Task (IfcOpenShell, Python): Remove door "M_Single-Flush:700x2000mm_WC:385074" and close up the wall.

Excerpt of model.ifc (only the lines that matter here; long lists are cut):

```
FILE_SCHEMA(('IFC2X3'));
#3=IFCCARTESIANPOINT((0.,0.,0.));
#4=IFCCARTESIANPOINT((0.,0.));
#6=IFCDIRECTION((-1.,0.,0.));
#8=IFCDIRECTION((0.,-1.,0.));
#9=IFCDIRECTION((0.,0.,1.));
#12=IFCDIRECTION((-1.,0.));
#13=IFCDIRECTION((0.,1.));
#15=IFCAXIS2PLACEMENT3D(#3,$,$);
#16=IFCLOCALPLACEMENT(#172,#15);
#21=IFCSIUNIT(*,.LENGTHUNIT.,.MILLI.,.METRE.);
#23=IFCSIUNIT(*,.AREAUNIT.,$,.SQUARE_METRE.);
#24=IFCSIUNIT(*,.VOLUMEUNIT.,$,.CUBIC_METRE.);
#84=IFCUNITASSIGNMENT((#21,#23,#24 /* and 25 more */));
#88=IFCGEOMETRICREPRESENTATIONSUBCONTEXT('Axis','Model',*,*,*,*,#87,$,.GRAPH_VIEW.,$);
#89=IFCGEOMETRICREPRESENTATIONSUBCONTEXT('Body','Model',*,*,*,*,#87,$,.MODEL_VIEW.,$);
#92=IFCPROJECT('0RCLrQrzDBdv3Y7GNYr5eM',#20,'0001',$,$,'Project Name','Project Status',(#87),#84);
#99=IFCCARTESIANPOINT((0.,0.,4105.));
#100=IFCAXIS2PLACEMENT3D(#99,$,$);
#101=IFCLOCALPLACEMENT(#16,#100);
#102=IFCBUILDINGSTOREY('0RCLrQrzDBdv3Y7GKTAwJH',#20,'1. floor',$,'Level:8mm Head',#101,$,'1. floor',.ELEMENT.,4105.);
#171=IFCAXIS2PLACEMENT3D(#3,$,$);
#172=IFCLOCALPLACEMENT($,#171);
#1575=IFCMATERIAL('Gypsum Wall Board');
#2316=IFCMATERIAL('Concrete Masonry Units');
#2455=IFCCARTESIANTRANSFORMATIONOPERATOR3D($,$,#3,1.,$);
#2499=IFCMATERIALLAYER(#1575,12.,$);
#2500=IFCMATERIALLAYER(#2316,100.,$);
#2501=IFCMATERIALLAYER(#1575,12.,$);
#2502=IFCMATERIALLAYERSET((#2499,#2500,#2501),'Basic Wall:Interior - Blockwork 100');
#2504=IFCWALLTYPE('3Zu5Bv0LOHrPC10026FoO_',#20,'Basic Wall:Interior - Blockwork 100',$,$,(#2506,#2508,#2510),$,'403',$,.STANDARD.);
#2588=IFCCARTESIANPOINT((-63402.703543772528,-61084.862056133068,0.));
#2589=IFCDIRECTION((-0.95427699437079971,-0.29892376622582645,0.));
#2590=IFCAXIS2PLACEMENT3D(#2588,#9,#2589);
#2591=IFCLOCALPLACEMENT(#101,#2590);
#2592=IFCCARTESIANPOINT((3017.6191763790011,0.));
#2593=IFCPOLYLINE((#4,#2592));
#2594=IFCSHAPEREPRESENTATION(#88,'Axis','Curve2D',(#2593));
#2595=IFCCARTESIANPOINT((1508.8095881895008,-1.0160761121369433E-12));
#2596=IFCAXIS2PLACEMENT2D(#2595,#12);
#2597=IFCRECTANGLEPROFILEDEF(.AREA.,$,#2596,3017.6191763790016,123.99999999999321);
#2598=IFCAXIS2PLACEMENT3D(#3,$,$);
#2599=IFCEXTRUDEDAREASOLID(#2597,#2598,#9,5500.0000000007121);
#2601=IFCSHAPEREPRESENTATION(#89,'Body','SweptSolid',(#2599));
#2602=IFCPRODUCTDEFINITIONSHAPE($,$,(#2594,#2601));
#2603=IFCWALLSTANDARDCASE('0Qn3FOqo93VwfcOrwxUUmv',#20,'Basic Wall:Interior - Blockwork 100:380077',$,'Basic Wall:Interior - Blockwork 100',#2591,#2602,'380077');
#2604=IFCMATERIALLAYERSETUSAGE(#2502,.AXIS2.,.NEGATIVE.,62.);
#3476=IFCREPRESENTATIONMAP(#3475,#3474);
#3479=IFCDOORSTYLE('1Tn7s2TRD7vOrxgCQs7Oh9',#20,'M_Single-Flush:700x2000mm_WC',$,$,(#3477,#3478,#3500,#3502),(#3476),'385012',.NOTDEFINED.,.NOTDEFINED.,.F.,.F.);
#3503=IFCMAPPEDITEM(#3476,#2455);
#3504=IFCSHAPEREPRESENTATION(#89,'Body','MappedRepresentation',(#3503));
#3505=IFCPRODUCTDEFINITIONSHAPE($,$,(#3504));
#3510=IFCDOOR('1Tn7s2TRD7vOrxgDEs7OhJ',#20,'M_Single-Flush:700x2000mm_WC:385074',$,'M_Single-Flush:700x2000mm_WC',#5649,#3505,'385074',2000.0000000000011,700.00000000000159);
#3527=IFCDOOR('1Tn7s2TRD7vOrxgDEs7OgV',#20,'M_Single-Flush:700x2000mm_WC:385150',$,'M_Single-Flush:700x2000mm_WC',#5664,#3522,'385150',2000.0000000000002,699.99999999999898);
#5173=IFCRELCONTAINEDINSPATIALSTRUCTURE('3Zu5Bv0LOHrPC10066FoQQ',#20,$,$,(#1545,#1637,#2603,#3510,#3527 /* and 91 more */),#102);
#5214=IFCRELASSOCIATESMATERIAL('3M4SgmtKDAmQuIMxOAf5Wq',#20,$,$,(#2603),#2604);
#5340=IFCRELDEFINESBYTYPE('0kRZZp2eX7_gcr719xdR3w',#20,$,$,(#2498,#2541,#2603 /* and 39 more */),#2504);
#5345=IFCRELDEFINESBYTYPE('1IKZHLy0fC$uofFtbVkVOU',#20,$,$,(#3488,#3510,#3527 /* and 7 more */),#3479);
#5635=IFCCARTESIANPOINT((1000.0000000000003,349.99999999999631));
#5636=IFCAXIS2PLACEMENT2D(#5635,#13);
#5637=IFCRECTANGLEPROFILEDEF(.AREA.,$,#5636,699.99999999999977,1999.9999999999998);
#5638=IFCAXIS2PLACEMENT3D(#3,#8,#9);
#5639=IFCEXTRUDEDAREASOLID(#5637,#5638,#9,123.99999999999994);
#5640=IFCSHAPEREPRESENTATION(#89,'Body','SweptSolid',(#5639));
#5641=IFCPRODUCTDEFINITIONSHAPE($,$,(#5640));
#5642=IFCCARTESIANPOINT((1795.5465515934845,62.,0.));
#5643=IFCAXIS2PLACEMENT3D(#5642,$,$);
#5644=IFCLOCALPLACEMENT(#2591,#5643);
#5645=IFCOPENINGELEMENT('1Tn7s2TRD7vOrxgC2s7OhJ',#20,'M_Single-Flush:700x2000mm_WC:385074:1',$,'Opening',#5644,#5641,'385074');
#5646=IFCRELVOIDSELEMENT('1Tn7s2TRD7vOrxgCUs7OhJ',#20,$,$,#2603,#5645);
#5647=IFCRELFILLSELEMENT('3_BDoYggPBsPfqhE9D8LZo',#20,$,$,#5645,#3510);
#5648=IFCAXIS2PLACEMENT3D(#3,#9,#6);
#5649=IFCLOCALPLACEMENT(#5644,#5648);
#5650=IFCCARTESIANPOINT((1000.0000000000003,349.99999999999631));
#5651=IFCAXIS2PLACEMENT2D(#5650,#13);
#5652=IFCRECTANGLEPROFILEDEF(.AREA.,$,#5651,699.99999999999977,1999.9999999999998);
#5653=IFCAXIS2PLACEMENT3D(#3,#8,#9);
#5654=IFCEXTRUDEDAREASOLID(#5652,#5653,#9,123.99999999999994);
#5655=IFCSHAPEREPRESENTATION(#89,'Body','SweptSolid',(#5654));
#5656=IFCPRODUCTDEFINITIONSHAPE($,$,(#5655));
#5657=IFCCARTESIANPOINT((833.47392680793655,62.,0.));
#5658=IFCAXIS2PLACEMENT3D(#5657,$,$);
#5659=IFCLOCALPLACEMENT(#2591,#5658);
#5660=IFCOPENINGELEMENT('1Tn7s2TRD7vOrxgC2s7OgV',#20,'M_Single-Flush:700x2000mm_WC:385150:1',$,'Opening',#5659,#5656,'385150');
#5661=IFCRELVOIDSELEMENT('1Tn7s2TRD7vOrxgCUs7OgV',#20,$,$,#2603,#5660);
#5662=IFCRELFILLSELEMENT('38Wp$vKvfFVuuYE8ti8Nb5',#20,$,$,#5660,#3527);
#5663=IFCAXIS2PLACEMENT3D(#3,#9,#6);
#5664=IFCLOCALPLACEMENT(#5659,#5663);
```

```python
import ifcopenshell
import ifcopenshell.api.feature
import ifcopenshell.api.root
import ifcopenshell.geom
import ifcopenshell.util.shape

model = ifcopenshell.open("model.ifc")
settings = ifcopenshell.geom.settings()


def volume(element):
    """Net volume in cubic metres, openings subtracted."""
    shape = ifcopenshell.geom.create_shape(settings, element)
    return ifcopenshell.util.shape.get_volume(shape.geometry)


door = model.by_guid("1Tn7s2TRD7vOrxgDEs7OhJ")
opening = door.FillsVoids[0].RelatingOpeningElement
wall = opening.VoidsElements[0].RelatingBuildingElement
before = volume(wall)

ifcopenshell.api.root.remove_product(model, product=door)
ifcopenshell.api.feature.remove_feature(model, feature=opening)

after = volume(wall)

print(f"wall volume {before:.3f} -> {after:.3f} m3")

model.write("model-out.ifc")
```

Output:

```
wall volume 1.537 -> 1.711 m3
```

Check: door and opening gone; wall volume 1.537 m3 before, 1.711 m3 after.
